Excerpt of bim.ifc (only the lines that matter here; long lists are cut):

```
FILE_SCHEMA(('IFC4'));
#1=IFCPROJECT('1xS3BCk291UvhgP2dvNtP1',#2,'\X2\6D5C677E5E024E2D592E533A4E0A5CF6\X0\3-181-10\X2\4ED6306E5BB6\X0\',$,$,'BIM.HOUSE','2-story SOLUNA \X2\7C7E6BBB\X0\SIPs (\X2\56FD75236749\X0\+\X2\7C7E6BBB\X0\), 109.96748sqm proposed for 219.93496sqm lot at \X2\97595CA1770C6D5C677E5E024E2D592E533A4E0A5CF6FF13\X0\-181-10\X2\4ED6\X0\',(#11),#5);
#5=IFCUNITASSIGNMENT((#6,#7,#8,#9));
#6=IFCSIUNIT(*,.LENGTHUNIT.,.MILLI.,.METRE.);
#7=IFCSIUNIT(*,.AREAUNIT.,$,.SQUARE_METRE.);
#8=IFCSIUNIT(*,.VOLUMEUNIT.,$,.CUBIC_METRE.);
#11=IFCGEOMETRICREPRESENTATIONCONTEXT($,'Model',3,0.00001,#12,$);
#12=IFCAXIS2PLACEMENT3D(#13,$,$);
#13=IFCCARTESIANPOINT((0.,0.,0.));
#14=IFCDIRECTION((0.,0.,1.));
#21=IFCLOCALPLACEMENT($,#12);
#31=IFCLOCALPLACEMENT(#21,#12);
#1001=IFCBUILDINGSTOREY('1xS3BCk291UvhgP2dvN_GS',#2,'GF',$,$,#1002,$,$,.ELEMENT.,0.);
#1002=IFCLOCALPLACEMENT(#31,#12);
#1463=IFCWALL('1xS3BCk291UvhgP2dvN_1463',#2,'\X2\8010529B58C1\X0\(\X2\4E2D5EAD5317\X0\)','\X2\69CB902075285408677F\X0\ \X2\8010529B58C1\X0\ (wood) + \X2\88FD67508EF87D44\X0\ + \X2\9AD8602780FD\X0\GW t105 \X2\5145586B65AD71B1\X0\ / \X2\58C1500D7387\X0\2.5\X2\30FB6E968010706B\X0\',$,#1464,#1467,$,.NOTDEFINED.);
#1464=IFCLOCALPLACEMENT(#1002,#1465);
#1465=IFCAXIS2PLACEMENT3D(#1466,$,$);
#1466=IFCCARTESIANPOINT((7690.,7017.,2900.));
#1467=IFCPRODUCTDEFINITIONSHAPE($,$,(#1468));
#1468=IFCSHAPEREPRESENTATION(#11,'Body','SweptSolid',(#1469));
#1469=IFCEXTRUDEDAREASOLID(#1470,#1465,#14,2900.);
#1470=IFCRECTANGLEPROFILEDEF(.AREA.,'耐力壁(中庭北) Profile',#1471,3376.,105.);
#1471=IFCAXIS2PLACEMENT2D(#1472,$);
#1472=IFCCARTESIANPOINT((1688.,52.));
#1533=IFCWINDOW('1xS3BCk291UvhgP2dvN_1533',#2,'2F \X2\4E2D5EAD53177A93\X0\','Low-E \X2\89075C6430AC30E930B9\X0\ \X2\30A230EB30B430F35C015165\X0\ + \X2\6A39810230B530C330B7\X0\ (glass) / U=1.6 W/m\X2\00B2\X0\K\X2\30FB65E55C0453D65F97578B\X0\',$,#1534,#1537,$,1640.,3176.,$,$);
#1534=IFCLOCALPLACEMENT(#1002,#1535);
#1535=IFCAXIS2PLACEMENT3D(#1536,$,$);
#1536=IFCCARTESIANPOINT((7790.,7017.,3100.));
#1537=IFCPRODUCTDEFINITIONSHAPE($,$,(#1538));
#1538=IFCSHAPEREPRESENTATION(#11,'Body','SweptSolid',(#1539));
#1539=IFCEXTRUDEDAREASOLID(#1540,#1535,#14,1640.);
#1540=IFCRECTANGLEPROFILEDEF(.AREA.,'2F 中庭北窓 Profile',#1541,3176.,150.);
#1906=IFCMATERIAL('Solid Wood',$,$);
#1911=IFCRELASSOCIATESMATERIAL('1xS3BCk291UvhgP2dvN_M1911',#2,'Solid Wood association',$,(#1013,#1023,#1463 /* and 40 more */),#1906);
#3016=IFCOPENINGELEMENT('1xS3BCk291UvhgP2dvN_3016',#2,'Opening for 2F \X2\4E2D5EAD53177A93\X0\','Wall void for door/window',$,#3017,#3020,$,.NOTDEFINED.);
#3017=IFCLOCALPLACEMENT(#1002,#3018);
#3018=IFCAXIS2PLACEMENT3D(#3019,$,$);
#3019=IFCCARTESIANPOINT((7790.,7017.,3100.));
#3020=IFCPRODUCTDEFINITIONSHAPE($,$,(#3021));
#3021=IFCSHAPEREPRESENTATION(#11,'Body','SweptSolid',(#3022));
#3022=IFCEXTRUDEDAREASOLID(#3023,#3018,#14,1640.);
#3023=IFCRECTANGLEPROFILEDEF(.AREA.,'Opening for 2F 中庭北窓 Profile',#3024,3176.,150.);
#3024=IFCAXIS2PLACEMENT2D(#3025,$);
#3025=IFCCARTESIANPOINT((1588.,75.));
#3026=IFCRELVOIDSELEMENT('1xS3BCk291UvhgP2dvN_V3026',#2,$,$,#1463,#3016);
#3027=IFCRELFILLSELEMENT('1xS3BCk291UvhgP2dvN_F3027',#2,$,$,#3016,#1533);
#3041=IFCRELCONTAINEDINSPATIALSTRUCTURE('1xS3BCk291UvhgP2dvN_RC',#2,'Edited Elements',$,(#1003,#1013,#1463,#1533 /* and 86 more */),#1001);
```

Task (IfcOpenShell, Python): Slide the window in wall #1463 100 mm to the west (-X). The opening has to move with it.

```python
import ifcopenshell
import ifcopenshell.api.geometry
import ifcopenshell.util.placement
import ifcopenshell.util.unit

model = ifcopenshell.open("bim.ifc")
unit_scale = ifcopenshell.util.unit.calculate_unit_scale(model)

window = model.by_id(1533)
opening = window.FillsVoids[0].RelatingOpeningElement
wall = opening.VoidsElements[0].RelatingBuildingElement

wall_matrix = ifcopenshell.util.placement.get_local_placement(wall.ObjectPlacement)
shift = wall_matrix[:3, 0] * -0.1 / unit_scale
before = ifcopenshell.util.placement.get_local_placement(window.ObjectPlacement)[:3, 3].copy()

# The window is not placed relative to its opening, so move both.
for product in (opening, window):
    matrix = ifcopenshell.util.placement.get_local_placement(product.ObjectPlacement)
    matrix[:3, 3] += shift
    ifcopenshell.api.geometry.edit_object_placement(model, product=product, matrix=matrix, is_si=False)

after = ifcopenshell.util.placement.get_local_placement(window.ObjectPlacement)[:3, 3]
print("window moved by", (after - before).round(3) + 0.0)

model.write("bim-out.ifc")
```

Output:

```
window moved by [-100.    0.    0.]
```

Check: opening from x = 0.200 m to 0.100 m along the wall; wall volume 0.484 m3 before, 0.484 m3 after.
